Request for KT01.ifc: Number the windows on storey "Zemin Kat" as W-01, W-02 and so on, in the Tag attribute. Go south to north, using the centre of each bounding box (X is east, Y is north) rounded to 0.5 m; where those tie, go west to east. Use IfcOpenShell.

First a look at what the model holds.

```python
import ifcopenshell
import ifcopenshell.util.element
import ifcopenshell.util.placement

model = ifcopenshell.open("KT01.ifc")
print(model.schema)
storey = next(s for s in model.by_type("IfcBuildingStorey") if s.Name == "Zemin Kat")
windows = [e for e in ifcopenshell.util.element.get_decomposition(storey) if e.is_a("IfcWindow")]
for e in sorted(windows, key=lambda e: e.id()):
    origin = ifcopenshell.util.placement.get_local_placement(e.ObjectPlacement)[:3, 3]
    print(e.id(), e.Tag, e.Name, origin.round(2) + 0.0, sep=" | ")
```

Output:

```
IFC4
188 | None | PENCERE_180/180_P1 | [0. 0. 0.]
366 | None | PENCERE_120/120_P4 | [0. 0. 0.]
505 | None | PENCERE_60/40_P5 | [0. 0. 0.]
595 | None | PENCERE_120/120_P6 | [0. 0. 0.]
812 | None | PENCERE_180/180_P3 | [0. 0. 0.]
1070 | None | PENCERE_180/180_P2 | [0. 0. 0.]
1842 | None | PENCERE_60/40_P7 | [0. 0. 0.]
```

```python
import ifcopenshell
import ifcopenshell.geom
import ifcopenshell.util.element
import ifcopenshell.util.shape

model = ifcopenshell.open("KT01.ifc")
settings = ifcopenshell.geom.settings()
settings.set("use-world-coords", True)


def centre(element):
    shape = ifcopenshell.geom.create_shape(settings, element)
    return ifcopenshell.util.shape.get_bbox_centroid(shape.geometry)


storey = next(s for s in model.by_type("IfcBuildingStorey") if s.Name == "Zemin Kat")
windows = [e for e in ifcopenshell.util.element.get_decomposition(storey) if e.is_a("IfcWindow")]

# Insertion points can sit at a corner or the storey origin, so sort by the geometry (in metres).
centres = {e: centre(e) for e in windows}
windows.sort(key=lambda e: (round(centres[e][1] / 0.5), centres[e][0]))

for i, e in enumerate(windows, start=1):
    number = f"W-{i:02d}"
    e.Tag = number
    print(e.id(), number)

model.write("KT01-out.ifc")
```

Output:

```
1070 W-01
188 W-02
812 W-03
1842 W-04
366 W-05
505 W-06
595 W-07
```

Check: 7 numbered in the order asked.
